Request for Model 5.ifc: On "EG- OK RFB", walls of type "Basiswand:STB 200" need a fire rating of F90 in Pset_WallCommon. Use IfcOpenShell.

First a look at what the model holds.

```python
import ifcopenshell
import ifcopenshell.util.element

model = ifcopenshell.open("Model 5.ifc")
print(model.schema)
storey = next(s for s in model.by_type("IfcBuildingStorey") if s.Name == "EG- OK RFB")
walls = [e for e in ifcopenshell.util.element.get_decomposition(storey) if e.is_a("IfcWall")]
seen = {}
for e in walls:
    element_type = ifcopenshell.util.element.get_type(e)
    key = (element_type.Name if element_type != e and element_type else None, ifcopenshell.util.element.get_pset(e, "Pset_WallCommon", "FireRating"))
    seen[key] = seen.get(key, 0) + 1
for (name, value), count in sorted(seen.items(), key=str):
    print(count, "x", name, "|", value)
```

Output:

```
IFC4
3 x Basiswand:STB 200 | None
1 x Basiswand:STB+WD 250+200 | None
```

```python
import ifcopenshell
import ifcopenshell.api.pset
import ifcopenshell.util.element

model = ifcopenshell.open("Model 5.ifc")

storey = next(s for s in model.by_type("IfcBuildingStorey") if s.Name == "EG- OK RFB")
walls = [e for e in ifcopenshell.util.element.get_decomposition(storey) if e.is_a("IfcWall")]

count = 0
for e in walls:
    element_type = ifcopenshell.util.element.get_type(e)
    if element_type in (None, e) or element_type.Name != "Basiswand:STB 200":
        continue
    # add_pset returns the element's existing set when there is one.
    pset = ifcopenshell.api.pset.add_pset(model, product=e, name="Pset_WallCommon")
    ifcopenshell.api.pset.edit_pset(model, pset=pset, properties={"FireRating": "F90"})
    count += 1

print(count, "walls updated")

model.write("Model 5_v2.ifc")
```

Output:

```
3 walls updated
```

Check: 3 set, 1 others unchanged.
